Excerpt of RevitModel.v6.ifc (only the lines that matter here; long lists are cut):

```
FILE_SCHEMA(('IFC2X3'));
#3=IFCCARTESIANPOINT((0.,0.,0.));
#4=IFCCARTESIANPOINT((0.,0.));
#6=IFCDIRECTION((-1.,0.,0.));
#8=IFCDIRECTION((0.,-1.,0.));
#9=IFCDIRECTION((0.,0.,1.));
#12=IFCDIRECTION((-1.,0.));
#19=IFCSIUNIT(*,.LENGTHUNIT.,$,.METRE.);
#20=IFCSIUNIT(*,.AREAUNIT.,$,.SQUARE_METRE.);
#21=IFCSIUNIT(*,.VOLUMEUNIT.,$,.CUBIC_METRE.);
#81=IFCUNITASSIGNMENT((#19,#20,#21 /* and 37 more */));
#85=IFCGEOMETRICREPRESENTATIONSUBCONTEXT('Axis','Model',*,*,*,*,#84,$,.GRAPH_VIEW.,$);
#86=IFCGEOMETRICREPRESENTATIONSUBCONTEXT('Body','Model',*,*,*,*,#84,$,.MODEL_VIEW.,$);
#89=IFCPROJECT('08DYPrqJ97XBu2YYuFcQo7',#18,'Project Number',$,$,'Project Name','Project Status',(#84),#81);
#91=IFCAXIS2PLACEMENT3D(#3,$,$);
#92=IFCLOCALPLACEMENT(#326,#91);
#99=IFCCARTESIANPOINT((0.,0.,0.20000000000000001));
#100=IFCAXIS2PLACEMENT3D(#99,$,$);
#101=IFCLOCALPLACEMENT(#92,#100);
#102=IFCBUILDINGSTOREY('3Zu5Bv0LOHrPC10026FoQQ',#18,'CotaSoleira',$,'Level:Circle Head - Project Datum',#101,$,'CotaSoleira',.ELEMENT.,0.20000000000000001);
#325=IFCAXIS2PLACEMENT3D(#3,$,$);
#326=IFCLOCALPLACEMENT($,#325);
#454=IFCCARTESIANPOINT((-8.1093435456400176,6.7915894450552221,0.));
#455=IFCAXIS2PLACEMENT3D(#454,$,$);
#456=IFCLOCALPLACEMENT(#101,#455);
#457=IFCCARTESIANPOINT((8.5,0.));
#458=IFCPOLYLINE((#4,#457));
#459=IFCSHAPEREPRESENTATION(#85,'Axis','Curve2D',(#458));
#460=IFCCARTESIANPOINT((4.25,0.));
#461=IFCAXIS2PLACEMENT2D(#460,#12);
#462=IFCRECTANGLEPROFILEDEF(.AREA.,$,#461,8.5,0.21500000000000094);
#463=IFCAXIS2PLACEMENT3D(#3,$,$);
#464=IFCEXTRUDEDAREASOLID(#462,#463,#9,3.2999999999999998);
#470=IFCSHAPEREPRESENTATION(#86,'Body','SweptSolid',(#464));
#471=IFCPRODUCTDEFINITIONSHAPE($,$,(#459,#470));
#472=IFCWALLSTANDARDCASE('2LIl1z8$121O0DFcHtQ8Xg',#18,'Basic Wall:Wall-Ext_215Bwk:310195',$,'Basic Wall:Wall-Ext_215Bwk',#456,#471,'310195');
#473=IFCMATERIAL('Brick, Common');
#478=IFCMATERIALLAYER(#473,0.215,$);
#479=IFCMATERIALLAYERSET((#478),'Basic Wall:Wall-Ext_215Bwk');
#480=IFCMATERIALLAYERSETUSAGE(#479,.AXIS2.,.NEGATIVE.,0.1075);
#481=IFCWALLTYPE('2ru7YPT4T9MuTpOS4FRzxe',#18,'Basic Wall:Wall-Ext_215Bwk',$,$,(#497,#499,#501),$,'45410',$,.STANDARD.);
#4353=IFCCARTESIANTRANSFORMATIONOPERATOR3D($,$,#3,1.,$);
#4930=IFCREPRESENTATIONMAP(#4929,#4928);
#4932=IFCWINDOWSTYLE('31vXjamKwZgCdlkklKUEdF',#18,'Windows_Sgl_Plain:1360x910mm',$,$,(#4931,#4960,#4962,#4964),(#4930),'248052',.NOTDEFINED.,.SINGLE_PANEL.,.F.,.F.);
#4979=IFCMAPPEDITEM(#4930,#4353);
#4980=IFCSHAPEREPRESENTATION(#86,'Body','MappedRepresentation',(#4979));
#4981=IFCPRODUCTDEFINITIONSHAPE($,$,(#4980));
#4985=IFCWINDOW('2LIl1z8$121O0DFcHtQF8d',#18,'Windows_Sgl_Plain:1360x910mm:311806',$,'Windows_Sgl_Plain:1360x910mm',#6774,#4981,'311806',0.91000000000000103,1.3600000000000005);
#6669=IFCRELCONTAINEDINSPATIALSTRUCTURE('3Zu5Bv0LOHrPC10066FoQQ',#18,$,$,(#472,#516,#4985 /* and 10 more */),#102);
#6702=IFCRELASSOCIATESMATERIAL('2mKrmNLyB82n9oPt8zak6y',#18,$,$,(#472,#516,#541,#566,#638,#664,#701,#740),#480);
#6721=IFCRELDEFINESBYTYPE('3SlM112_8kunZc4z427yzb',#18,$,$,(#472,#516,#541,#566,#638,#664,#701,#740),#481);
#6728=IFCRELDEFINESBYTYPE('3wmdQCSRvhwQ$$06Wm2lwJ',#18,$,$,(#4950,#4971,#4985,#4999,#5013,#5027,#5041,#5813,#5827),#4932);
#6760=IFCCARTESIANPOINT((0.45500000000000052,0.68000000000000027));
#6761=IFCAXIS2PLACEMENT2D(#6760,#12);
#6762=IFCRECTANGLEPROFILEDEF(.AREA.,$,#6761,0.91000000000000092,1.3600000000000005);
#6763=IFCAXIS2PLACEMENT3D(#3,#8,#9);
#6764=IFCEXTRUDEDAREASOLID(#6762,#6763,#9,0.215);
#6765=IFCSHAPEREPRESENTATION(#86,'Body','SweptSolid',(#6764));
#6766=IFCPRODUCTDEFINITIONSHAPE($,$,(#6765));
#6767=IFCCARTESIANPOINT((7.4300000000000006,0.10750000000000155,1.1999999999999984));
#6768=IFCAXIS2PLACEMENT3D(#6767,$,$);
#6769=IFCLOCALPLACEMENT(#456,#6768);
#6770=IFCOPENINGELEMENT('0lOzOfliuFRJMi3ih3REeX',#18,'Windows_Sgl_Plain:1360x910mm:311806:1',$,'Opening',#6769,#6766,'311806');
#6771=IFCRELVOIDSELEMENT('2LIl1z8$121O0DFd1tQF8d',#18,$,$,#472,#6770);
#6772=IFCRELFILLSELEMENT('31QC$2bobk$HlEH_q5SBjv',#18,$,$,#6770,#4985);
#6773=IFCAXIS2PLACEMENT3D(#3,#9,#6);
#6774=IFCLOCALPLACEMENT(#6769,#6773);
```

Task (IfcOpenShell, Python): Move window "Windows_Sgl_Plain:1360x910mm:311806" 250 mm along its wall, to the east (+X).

```python
import ifcopenshell
import ifcopenshell.api.geometry
import ifcopenshell.util.placement

model = ifcopenshell.open("RevitModel.v6.ifc")

window = model.by_guid("2LIl1z8$121O0DFcHtQF8d")
opening = window.FillsVoids[0].RelatingOpeningElement
wall = opening.VoidsElements[0].RelatingBuildingElement

wall_matrix = ifcopenshell.util.placement.get_local_placement(wall.ObjectPlacement)
shift = wall_matrix[:3, 0] * 0.25
before = ifcopenshell.util.placement.get_local_placement(window.ObjectPlacement)[:3, 3].copy()

# The window is placed relative to its opening, so it follows when the opening moves.
matrix = ifcopenshell.util.placement.get_local_placement(opening.ObjectPlacement)
matrix[:3, 3] += shift
ifcopenshell.api.geometry.edit_object_placement(
    model, product=opening, matrix=matrix, is_si=False, should_transform_children=True
)

after = ifcopenshell.util.placement.get_local_placement(window.ObjectPlacement)[:3, 3]
print("window moved by", (after - before).round(3) + 0.0)

model.write("RevitModel.v6_v2.ifc")
```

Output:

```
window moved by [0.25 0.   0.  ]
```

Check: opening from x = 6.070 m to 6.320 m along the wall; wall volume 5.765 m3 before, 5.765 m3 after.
